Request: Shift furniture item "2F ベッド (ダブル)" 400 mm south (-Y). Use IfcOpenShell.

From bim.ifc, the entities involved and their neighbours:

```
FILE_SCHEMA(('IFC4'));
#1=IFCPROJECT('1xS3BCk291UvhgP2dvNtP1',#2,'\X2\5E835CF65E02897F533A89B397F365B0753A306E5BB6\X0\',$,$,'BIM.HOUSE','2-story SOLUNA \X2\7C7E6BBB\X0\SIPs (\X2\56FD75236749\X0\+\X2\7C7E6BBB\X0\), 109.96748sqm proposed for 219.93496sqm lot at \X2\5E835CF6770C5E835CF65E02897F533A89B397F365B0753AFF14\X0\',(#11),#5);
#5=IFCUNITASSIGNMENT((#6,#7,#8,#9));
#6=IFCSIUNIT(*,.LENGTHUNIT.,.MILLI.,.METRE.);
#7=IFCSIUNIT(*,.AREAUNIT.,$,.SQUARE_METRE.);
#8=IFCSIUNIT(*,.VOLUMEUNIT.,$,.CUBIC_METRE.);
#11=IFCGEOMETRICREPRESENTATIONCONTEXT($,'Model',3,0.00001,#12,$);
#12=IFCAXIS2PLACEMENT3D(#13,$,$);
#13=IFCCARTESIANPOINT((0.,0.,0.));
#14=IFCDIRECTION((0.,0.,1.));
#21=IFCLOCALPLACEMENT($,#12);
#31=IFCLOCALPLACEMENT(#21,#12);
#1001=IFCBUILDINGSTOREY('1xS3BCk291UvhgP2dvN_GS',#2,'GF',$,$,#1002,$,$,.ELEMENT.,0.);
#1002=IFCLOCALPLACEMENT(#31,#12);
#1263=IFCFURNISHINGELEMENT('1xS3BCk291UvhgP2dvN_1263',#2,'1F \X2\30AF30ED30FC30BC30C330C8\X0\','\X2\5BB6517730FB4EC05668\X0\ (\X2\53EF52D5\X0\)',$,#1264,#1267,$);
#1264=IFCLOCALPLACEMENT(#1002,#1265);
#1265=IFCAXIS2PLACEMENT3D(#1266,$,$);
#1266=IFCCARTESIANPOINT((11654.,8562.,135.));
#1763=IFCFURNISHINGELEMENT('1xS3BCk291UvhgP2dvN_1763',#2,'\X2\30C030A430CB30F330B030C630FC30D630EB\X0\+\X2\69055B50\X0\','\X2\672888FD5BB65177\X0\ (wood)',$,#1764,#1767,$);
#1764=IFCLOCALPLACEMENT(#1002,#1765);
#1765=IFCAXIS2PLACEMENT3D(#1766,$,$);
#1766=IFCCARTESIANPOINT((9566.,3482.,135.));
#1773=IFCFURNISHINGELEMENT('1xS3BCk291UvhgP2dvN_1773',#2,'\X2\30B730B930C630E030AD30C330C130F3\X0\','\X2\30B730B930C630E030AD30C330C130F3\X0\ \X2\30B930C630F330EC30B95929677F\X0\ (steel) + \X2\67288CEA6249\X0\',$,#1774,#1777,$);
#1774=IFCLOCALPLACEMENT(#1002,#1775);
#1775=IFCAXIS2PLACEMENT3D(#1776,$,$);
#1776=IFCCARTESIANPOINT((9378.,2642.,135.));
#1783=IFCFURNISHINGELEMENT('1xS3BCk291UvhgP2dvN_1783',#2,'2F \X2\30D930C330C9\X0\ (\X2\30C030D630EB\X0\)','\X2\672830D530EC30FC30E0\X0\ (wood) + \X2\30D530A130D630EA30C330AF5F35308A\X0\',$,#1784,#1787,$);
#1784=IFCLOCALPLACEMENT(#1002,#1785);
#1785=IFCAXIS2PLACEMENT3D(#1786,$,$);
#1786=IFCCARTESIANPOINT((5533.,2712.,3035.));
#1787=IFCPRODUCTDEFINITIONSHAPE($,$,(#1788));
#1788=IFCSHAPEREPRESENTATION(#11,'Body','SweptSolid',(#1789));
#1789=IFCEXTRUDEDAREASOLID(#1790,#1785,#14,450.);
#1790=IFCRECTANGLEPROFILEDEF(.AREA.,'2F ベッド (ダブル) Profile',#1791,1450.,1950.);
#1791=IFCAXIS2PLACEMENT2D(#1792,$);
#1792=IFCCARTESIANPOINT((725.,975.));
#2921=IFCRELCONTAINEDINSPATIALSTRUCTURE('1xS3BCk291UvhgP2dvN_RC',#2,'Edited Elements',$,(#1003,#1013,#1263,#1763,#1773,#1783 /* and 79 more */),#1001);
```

```python
import ifcopenshell
import ifcopenshell.api.geometry
import ifcopenshell.util.placement

model = ifcopenshell.open("bim.ifc")

item = model.by_guid("1xS3BCk291UvhgP2dvN_1783")
matrix = ifcopenshell.util.placement.get_local_placement(item.ObjectPlacement)
matrix[1, 3] -= 400.0
ifcopenshell.api.geometry.edit_object_placement(model, product=item, matrix=matrix, is_si=False)

print(ifcopenshell.util.placement.get_local_placement(item.ObjectPlacement).round(3) + 0.0)

model.write("bim_rev.ifc")
```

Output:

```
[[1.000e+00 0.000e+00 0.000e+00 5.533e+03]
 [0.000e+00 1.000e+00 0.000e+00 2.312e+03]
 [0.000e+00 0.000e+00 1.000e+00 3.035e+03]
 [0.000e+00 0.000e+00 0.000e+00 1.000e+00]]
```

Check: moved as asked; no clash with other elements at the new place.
